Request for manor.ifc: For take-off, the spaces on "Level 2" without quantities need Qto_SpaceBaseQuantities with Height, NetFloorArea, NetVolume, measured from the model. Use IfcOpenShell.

First a look at what the model holds.

```python
import ifcopenshell
import ifcopenshell.util.element
import ifcopenshell.util.unit

model = ifcopenshell.open("manor.ifc")
print(model.schema)
for unit_type in ("LENGTHUNIT", "AREAUNIT", "VOLUMEUNIT"):
    print(unit_type, ifcopenshell.util.unit.calculate_unit_scale(model, unit_type))
storey = next(s for s in model.by_type("IfcBuildingStorey") if s.Name == "Level 2")
spaces = [e for e in ifcopenshell.util.element.get_decomposition(storey) if e.is_a("IfcSpace")]
for e in sorted(spaces, key=lambda e: e.id()):
    print(e.id(), e.is_a(), e.Name, list(ifcopenshell.util.element.get_psets(e, qtos_only=True)), sep=" | ")
```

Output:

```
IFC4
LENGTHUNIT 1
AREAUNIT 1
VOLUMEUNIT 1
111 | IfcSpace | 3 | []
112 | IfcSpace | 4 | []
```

```python
import ifcopenshell
import ifcopenshell.api.pset
import ifcopenshell.geom
import ifcopenshell.util.element
import ifcopenshell.util.shape
import ifcopenshell.util.unit

model = ifcopenshell.open("manor.ifc")
unit_scale = ifcopenshell.util.unit.calculate_unit_scale(model)
area_scale = ifcopenshell.util.unit.calculate_unit_scale(model, "AREAUNIT")
volume_scale = ifcopenshell.util.unit.calculate_unit_scale(model, "VOLUMEUNIT")
settings = ifcopenshell.geom.settings()

storey = next(s for s in model.by_type("IfcBuildingStorey") if s.Name == "Level 2")
spaces = [e for e in ifcopenshell.util.element.get_decomposition(storey) if e.is_a("IfcSpace")]

for e in sorted(spaces, key=lambda e: e.id()):
    if ifcopenshell.util.element.get_psets(e, qtos_only=True, should_inherit=False):
        continue
    # Geometry comes back in metres, in the element's own axes.
    shape = ifcopenshell.geom.create_shape(settings, e)
    values = {
        "Height": ifcopenshell.util.shape.get_z(shape.geometry) / unit_scale,
        "NetFloorArea": ifcopenshell.util.shape.get_footprint_area(shape.geometry) / area_scale,
        "NetVolume": ifcopenshell.util.shape.get_volume(shape.geometry) / volume_scale,
    }
    qto = ifcopenshell.api.pset.add_qto(model, product=e, name="Qto_SpaceBaseQuantities")
    ifcopenshell.api.pset.edit_qto(model, qto=qto, properties=values)
    print(e.id(), {k: round(v, 3) for k, v in values.items()})

model.write("manor-out.ifc")
```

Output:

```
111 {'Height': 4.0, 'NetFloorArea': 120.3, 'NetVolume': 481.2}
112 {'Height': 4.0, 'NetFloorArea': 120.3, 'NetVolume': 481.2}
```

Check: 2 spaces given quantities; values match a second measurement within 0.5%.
